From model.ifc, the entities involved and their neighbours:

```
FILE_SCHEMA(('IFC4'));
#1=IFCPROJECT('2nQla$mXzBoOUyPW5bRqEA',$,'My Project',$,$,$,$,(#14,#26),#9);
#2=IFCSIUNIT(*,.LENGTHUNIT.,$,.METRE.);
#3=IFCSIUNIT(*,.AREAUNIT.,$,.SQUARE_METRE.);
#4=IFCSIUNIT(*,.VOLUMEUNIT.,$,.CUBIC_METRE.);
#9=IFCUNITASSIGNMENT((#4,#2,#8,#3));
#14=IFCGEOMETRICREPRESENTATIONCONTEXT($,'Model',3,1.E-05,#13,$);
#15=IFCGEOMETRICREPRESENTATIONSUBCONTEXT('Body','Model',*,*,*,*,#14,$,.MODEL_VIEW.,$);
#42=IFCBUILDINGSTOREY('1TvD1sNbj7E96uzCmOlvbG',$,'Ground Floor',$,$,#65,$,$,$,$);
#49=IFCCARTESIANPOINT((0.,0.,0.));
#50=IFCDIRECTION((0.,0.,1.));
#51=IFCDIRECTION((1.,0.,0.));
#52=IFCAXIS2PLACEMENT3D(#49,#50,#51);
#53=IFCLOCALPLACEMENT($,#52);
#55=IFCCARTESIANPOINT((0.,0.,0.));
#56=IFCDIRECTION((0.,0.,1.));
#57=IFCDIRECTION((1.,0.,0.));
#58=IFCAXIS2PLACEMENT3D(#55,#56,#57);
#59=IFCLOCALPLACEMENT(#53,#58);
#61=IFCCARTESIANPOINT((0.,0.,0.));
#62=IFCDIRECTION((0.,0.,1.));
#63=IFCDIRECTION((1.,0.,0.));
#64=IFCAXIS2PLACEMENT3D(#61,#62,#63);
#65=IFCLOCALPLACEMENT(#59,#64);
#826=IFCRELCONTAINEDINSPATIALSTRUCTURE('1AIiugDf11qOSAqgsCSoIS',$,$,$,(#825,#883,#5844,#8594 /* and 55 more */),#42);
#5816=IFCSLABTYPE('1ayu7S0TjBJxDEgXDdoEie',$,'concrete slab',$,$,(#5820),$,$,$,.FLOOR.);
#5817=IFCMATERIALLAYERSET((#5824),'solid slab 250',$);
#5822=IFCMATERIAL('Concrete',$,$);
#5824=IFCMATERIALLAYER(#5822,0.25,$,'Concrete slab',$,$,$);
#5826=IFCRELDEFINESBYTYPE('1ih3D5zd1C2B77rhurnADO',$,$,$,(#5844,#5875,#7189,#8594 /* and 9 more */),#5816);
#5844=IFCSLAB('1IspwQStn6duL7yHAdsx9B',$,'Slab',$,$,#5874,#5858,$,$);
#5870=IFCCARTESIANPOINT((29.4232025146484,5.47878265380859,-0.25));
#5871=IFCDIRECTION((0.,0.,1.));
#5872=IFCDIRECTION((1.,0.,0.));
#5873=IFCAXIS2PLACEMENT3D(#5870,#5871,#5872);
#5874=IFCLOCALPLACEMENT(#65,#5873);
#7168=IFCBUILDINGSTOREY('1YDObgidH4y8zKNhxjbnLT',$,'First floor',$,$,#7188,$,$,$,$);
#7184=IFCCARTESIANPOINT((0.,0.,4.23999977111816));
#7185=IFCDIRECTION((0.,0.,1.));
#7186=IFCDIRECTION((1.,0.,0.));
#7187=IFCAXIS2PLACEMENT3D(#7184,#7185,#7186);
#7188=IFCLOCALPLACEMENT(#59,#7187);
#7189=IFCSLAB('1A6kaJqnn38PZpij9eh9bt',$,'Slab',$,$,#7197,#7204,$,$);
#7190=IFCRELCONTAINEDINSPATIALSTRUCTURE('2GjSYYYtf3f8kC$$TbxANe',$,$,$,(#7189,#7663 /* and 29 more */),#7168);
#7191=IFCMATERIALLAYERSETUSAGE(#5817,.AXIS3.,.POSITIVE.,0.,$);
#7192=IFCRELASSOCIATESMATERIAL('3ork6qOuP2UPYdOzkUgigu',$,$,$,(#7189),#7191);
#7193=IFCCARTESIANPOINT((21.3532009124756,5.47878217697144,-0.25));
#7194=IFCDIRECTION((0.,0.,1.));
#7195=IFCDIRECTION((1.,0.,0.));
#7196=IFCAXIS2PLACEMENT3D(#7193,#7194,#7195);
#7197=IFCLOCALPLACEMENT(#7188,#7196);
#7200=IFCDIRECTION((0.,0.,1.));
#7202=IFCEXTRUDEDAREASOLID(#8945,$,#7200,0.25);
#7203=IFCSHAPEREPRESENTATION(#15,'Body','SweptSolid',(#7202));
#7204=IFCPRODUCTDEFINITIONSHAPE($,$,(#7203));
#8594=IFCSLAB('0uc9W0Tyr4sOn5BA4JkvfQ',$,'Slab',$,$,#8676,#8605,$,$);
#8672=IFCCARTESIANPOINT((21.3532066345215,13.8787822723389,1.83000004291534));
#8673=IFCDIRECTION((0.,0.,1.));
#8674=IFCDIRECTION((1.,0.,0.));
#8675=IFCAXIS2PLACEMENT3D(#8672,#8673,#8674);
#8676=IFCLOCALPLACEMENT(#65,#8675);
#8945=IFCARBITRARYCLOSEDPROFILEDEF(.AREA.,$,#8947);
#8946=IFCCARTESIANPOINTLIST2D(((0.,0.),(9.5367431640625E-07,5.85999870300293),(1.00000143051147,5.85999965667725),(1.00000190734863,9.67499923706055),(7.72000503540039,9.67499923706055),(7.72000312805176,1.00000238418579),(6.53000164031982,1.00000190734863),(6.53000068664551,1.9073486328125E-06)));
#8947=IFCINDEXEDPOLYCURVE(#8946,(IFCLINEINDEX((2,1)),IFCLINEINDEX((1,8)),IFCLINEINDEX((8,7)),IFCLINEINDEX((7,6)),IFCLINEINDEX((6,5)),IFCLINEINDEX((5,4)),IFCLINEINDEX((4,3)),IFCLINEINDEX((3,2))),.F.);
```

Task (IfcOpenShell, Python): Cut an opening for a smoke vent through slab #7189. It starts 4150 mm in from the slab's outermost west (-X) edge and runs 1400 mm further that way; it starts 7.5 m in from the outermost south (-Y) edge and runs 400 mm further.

```python
import numpy as np
import ifcopenshell
import ifcopenshell.api.feature
import ifcopenshell.api.geometry
import ifcopenshell.api.root
import ifcopenshell.geom
import ifcopenshell.util.placement
import ifcopenshell.util.representation
import ifcopenshell.util.shape
import ifcopenshell.util.unit

model = ifcopenshell.open("model.ifc")
unit_scale = ifcopenshell.util.unit.calculate_unit_scale(model)
settings = ifcopenshell.geom.settings()


def volume(element):
    """Net volume in cubic metres, openings subtracted."""
    shape = ifcopenshell.geom.create_shape(settings, element)
    return ifcopenshell.util.shape.get_volume(shape.geometry)


slab = model.by_guid("1A6kaJqnn38PZpij9eh9bt")
before = volume(slab)

# Extent in the slab's own axes, in metres. The edges named are its -X and -Y sides.
slab_shape = ifcopenshell.geom.create_shape(settings, slab)
vertices = ifcopenshell.util.shape.get_vertices(slab_shape.geometry)
x_min, y_min, bottom = vertices.min(axis=0)
top = vertices[:, 2].max()

opening = ifcopenshell.api.root.create_entity(model, ifc_class="IfcOpeningElement", name="Smoke vent opening", predefined_type="OPENING")
context = ifcopenshell.util.representation.get_context(model, "Model", "Body", "MODEL_VIEW")
width, depth = 1.4, 0.4
outline = [(0.0, 0.0), (width, 0.0), (width, depth), (0.0, depth), (0.0, 0.0)]
# Overshoot both faces by 50 mm so the cut is clean.
shape = ifcopenshell.api.geometry.add_slab_representation(
    model, context=context, depth=top - bottom + 0.1, polyline=outline
)
ifcopenshell.api.geometry.assign_representation(model, product=opening, representation=shape)

matrix = ifcopenshell.util.placement.get_local_placement(slab.ObjectPlacement)
matrix[:, 3] = matrix @ np.append(np.array([x_min + 4.15, y_min + 7.5, bottom - 0.05]) / unit_scale, 1.0)
ifcopenshell.api.geometry.edit_object_placement(model, product=opening, matrix=matrix, is_si=False)
ifcopenshell.api.feature.add_feature(model, feature=opening, element=slab)

after = volume(slab)

print(f"slab volume {before:.3f} -> {after:.3f} m3")

model.write("model_updated.ifc")
```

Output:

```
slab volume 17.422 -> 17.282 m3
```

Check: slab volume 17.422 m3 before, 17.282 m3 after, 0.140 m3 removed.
